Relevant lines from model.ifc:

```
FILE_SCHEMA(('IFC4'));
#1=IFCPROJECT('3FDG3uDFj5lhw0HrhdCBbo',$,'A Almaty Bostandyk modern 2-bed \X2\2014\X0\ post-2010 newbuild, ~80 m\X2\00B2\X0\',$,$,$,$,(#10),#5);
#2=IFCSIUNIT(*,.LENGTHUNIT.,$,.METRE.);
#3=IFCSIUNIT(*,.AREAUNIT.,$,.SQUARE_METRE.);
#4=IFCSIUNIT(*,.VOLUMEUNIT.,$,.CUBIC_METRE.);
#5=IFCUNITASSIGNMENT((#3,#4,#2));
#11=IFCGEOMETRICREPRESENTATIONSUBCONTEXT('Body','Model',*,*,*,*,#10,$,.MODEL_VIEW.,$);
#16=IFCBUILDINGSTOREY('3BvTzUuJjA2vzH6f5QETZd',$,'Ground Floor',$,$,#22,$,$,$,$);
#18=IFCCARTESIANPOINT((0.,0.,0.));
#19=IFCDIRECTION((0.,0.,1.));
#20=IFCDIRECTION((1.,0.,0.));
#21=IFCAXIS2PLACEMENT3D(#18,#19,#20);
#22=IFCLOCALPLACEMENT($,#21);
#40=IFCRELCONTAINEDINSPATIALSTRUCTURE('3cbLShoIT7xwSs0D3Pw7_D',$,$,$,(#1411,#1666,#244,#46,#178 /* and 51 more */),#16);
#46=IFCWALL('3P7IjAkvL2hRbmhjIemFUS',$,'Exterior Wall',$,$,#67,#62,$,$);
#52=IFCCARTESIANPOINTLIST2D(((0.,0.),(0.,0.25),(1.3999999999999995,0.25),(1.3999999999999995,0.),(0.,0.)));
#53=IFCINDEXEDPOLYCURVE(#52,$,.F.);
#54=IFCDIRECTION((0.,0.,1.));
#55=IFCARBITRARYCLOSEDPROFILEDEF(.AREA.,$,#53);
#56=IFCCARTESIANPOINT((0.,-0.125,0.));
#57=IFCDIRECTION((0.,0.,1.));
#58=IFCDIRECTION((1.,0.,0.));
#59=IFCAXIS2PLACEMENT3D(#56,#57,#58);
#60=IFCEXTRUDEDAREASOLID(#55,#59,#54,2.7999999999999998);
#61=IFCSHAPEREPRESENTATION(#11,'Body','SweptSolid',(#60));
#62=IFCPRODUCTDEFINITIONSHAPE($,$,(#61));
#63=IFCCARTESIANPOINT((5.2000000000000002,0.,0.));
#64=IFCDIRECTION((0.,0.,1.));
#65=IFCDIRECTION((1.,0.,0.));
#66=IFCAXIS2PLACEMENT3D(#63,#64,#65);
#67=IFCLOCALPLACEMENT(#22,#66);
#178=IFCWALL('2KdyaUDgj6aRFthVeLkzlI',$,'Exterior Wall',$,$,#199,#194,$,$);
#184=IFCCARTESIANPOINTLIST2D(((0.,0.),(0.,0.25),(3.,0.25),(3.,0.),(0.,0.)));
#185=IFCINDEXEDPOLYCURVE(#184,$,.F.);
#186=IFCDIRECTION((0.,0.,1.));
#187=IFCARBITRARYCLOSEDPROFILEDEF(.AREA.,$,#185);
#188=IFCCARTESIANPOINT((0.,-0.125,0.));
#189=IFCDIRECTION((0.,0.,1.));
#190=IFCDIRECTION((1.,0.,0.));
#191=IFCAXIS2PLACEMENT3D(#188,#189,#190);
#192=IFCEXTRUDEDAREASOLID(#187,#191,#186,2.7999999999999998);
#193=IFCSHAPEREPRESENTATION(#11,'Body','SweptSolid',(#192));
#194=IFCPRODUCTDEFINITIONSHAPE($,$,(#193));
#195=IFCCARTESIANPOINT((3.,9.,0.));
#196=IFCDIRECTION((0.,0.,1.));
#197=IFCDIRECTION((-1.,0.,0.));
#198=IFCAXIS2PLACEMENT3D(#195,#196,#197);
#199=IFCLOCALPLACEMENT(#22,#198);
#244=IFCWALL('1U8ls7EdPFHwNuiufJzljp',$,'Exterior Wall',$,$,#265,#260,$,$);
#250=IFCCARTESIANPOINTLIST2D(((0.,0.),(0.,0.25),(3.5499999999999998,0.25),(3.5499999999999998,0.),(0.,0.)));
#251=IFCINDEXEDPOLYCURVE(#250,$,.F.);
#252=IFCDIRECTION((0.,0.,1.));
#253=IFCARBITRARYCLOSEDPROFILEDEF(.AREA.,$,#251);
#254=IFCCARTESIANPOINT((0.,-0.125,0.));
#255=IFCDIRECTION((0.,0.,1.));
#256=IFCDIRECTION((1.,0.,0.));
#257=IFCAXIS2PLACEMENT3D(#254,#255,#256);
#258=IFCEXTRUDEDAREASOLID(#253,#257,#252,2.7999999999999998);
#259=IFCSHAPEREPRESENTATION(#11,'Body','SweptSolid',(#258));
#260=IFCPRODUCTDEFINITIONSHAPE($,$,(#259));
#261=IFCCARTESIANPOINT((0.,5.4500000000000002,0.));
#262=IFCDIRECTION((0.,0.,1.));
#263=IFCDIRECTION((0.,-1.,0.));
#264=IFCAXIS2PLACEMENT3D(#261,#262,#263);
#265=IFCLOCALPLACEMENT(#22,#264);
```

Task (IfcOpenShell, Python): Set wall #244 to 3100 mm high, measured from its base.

```python
import ifcopenshell
import ifcopenshell.geom
import ifcopenshell.util.representation
import ifcopenshell.util.shape
import ifcopenshell.util.unit

model = ifcopenshell.open("model.ifc")
unit_scale = ifcopenshell.util.unit.calculate_unit_scale(model)
settings = ifcopenshell.geom.settings()


def volume(element):
    """Net volume in cubic metres, openings subtracted."""
    shape = ifcopenshell.geom.create_shape(settings, element)
    return ifcopenshell.util.shape.get_volume(shape.geometry)


wall = model.by_guid("1U8ls7EdPFHwNuiufJzljp")
before = volume(wall)

body = ifcopenshell.util.representation.get_representation(wall, "Model", "Body")
solid = body.Items[0]
old_height = solid.Depth
solid.Depth = 3.1 / unit_scale
after = volume(wall)

print(f"height {old_height:g} -> {solid.Depth:g}, volume {before:.3f} -> {after:.3f} m3")

model.write("model_updated.ifc")
```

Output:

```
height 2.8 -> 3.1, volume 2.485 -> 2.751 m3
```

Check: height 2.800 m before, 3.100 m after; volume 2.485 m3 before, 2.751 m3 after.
